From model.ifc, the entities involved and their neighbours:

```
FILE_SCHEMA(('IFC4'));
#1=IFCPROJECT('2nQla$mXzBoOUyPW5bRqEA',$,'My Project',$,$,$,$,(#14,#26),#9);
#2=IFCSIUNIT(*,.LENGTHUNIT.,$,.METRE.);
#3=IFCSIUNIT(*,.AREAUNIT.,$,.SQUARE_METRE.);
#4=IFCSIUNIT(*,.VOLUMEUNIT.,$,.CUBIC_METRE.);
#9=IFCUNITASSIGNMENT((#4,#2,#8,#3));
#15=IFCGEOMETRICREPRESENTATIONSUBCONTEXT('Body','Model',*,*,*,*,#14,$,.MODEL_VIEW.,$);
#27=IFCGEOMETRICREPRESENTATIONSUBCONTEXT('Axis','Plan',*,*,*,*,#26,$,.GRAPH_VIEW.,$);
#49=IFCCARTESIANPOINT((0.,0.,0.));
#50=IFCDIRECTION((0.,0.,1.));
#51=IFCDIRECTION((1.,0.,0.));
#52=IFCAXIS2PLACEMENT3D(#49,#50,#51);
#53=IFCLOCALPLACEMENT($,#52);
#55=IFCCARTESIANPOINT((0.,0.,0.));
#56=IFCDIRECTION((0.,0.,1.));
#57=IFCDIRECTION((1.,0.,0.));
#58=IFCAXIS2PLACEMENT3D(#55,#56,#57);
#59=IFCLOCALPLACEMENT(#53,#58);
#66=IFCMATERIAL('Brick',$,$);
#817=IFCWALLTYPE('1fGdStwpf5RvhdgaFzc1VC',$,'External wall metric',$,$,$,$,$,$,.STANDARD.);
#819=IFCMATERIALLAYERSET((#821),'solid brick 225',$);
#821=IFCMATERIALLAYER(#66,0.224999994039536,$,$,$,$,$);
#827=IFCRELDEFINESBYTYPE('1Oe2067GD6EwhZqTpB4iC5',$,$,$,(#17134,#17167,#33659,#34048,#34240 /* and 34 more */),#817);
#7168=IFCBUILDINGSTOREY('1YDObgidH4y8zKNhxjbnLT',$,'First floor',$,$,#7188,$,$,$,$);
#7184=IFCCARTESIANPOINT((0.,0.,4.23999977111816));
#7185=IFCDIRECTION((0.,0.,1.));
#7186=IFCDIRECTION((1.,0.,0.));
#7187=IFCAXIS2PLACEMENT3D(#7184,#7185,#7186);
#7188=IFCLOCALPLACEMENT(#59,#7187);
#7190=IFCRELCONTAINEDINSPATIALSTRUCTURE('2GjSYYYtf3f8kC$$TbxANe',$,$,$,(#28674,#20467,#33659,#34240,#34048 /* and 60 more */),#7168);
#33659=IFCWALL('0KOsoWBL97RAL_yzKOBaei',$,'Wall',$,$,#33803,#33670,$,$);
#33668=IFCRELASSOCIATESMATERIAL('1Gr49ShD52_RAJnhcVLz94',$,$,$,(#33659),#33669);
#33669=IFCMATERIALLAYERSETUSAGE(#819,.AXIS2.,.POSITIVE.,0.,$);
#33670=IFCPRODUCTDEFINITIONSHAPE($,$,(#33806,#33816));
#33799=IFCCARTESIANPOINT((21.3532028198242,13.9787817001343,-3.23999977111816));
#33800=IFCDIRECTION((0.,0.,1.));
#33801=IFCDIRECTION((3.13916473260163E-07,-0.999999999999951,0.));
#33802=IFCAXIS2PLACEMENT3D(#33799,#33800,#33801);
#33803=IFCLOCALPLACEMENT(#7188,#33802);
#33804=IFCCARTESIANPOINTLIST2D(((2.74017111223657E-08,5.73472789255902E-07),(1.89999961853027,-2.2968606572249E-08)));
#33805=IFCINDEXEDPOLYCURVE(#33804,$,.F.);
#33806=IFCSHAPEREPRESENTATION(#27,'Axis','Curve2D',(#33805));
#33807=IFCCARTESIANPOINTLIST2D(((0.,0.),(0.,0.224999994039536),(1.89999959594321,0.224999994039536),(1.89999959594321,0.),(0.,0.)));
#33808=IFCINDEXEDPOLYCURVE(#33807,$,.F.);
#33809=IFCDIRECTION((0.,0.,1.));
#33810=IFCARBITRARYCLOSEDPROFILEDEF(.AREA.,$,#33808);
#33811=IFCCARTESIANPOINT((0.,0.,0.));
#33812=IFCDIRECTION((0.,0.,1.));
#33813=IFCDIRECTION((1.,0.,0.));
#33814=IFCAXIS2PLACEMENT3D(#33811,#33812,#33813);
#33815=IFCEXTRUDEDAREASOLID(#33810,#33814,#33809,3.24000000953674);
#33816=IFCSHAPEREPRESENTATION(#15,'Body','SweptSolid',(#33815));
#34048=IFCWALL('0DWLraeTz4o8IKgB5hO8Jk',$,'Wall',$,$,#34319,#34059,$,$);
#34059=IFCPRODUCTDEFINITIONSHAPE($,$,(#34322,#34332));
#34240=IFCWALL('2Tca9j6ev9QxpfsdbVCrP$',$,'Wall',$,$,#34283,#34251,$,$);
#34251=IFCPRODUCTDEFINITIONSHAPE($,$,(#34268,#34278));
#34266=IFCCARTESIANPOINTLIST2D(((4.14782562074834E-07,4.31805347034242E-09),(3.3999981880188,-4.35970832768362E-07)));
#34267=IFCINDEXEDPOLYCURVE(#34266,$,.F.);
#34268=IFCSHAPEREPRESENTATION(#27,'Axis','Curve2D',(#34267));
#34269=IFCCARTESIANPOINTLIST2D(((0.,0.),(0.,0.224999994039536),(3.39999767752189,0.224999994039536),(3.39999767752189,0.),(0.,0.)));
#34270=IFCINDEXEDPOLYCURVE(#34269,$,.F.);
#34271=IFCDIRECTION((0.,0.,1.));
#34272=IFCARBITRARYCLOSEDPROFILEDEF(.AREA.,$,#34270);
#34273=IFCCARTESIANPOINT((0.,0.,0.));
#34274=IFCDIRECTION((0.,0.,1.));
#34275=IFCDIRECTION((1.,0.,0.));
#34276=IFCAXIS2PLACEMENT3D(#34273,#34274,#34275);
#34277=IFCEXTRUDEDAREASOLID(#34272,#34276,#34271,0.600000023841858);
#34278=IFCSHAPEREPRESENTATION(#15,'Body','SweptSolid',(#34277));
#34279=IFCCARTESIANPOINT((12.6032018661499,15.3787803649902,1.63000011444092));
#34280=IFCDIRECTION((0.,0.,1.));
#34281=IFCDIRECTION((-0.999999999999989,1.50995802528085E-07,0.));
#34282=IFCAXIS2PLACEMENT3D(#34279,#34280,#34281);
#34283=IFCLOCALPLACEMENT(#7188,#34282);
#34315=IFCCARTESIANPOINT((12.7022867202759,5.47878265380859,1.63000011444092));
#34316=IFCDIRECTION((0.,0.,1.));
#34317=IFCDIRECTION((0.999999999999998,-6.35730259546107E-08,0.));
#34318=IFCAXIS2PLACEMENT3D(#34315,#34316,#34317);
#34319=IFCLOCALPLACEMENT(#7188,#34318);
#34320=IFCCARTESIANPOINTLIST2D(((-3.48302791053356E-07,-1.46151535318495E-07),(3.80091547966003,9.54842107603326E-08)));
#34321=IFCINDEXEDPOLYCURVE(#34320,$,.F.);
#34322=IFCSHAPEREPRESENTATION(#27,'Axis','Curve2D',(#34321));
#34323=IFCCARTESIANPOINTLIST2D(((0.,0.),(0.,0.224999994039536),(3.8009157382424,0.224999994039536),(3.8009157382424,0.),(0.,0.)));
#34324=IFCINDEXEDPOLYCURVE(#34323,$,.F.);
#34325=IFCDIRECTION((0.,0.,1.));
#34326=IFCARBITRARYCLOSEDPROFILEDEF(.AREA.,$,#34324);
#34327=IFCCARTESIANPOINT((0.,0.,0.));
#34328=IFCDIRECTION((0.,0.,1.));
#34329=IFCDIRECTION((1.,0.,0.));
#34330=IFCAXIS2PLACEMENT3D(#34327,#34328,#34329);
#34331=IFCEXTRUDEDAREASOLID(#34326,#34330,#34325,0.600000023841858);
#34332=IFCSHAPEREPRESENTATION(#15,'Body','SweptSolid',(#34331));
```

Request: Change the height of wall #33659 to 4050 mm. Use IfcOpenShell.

```python
import ifcopenshell
import ifcopenshell.geom
import ifcopenshell.util.representation
import ifcopenshell.util.shape
import ifcopenshell.util.unit

model = ifcopenshell.open("model.ifc")
unit_scale = ifcopenshell.util.unit.calculate_unit_scale(model)
settings = ifcopenshell.geom.settings()


def volume(element):
    """Net volume in cubic metres, openings subtracted."""
    shape = ifcopenshell.geom.create_shape(settings, element)
    return ifcopenshell.util.shape.get_volume(shape.geometry)


wall = model.by_id(33659)
before = volume(wall)

body = ifcopenshell.util.representation.get_representation(wall, "Model", "Body")
solid = body.Items[0]
old_height = solid.Depth
solid.Depth = 4.05 / unit_scale
after = volume(wall)

print(f"height {old_height:g} -> {solid.Depth:g}, volume {before:.3f} -> {after:.3f} m3")

model.write("model-out.ifc")
```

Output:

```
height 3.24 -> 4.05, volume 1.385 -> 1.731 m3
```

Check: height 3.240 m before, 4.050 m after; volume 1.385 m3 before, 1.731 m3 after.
